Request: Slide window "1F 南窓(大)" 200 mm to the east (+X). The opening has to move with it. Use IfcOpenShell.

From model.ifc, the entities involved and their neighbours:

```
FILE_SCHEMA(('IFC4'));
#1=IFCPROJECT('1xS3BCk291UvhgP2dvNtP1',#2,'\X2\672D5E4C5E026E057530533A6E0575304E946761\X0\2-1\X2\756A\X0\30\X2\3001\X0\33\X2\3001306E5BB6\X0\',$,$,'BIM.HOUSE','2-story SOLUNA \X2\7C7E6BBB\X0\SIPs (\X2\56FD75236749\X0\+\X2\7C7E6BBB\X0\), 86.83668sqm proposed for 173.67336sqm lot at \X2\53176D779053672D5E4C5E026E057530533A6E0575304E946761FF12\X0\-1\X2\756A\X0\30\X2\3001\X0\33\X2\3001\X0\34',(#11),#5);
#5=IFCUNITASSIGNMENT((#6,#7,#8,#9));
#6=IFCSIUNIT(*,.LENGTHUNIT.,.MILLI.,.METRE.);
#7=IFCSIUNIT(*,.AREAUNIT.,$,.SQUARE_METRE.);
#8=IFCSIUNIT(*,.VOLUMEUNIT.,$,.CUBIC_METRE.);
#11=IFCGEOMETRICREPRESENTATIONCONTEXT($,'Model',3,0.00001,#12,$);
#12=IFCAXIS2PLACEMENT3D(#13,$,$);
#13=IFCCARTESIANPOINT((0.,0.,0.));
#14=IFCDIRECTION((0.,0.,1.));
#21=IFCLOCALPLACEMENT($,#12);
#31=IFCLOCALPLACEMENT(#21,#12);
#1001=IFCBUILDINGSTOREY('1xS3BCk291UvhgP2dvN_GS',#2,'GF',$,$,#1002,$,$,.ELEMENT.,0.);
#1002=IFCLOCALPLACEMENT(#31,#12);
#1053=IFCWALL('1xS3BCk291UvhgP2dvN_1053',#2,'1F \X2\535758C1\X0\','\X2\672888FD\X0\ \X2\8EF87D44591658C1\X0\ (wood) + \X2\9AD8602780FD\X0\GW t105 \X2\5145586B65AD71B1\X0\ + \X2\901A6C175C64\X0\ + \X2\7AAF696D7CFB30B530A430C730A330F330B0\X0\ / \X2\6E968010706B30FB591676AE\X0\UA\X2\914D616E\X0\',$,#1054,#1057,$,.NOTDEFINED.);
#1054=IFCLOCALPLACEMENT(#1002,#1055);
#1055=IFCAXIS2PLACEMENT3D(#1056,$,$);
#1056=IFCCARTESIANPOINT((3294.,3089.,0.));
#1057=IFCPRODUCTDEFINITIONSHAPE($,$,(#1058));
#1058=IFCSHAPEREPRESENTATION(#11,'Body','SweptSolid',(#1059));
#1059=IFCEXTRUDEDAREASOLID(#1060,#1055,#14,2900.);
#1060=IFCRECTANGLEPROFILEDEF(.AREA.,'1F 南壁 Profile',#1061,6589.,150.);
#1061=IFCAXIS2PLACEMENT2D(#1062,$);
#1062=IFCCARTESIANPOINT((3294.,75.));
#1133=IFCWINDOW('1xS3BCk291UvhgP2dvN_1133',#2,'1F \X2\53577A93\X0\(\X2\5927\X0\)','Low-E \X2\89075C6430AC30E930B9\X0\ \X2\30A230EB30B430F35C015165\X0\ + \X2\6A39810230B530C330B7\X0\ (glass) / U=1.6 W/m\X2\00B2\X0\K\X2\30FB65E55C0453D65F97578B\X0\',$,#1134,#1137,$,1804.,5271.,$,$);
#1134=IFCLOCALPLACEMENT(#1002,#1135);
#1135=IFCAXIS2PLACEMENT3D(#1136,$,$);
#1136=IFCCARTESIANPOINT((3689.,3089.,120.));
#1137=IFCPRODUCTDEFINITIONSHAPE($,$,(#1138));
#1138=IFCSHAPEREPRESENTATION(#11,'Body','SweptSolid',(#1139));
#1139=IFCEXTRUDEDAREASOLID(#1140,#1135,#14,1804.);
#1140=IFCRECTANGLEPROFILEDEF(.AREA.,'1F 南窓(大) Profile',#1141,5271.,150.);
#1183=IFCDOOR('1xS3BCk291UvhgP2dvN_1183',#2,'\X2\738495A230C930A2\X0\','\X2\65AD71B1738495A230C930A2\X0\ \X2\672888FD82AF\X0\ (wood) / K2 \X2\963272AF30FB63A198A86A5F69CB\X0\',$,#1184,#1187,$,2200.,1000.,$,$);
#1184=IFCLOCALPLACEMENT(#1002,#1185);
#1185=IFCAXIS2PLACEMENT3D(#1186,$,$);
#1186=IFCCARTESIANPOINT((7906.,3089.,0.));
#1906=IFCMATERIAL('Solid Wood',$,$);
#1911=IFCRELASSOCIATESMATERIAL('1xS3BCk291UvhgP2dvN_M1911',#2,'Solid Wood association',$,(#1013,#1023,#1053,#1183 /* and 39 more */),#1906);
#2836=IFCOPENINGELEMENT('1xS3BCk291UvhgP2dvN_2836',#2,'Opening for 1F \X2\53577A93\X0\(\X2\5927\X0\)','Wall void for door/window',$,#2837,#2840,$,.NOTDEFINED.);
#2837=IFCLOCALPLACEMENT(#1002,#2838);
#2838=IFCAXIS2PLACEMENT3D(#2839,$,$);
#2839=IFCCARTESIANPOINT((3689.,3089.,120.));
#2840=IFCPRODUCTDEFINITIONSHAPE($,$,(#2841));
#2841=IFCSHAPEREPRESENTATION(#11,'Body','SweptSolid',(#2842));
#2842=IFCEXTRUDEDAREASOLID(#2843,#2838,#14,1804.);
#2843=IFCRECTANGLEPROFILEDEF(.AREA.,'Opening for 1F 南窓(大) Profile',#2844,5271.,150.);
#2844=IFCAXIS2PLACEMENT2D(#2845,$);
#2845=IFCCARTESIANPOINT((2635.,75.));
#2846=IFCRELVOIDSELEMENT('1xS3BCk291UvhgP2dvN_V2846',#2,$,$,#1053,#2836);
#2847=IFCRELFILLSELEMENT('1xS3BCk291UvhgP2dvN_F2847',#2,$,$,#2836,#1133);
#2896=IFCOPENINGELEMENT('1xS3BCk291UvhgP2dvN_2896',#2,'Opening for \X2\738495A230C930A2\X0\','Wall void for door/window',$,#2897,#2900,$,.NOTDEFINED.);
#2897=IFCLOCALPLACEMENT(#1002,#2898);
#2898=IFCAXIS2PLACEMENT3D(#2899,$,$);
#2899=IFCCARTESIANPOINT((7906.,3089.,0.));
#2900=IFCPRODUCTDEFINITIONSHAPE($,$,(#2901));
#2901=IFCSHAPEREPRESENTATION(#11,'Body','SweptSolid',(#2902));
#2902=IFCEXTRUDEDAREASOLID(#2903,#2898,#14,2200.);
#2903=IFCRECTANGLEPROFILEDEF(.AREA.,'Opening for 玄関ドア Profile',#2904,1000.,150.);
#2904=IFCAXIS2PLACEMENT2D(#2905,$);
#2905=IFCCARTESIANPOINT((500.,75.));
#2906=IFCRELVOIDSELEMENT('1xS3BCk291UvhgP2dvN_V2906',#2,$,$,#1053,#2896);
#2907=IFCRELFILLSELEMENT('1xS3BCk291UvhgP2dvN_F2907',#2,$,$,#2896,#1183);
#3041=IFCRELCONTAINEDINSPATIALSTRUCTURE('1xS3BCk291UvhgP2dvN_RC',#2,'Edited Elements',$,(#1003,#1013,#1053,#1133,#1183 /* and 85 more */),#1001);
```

```python
import ifcopenshell
import ifcopenshell.api.geometry
import ifcopenshell.util.placement
import ifcopenshell.util.unit

model = ifcopenshell.open("model.ifc")
unit_scale = ifcopenshell.util.unit.calculate_unit_scale(model)

window = model.by_guid("1xS3BCk291UvhgP2dvN_1133")
opening = window.FillsVoids[0].RelatingOpeningElement
wall = opening.VoidsElements[0].RelatingBuildingElement

wall_matrix = ifcopenshell.util.placement.get_local_placement(wall.ObjectPlacement)
shift = wall_matrix[:3, 0] * 0.2 / unit_scale
before = ifcopenshell.util.placement.get_local_placement(window.ObjectPlacement)[:3, 3].copy()

# The window is not placed relative to its opening, so move both.
for product in (opening, window):
    matrix = ifcopenshell.util.placement.get_local_placement(product.ObjectPlacement)
    matrix[:3, 3] += shift
    ifcopenshell.api.geometry.edit_object_placement(model, product=product, matrix=matrix, is_si=False)

after = ifcopenshell.util.placement.get_local_placement(window.ObjectPlacement)[:3, 3]
print("window moved by", (after - before).round(3) + 0.0)

model.write("model_v2.ifc")
```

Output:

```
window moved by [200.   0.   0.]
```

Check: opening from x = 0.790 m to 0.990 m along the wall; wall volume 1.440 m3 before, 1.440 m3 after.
